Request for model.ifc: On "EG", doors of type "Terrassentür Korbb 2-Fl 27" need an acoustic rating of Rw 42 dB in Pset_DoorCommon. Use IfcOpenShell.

First a look at what the model holds.

```python
import ifcopenshell
import ifcopenshell.util.element

model = ifcopenshell.open("model.ifc")
print(model.schema)
storey = next(s for s in model.by_type("IfcBuildingStorey") if s.Name == "EG")
doors = [e for e in ifcopenshell.util.element.get_decomposition(storey) if e.is_a("IfcDoor")]
seen = {}
for e in doors:
    element_type = ifcopenshell.util.element.get_type(e)
    key = (element_type.Name if element_type != e and element_type else None, ifcopenshell.util.element.get_pset(e, "Pset_DoorCommon", "AcousticRating"))
    seen[key] = seen.get(key, 0) + 1
for (name, value), count in sorted(seen.items(), key=str):
    print(count, "x", name, "|", value)
```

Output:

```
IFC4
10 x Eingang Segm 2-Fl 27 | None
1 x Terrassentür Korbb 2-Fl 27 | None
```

```python
import ifcopenshell
import ifcopenshell.api.pset
import ifcopenshell.util.element

model = ifcopenshell.open("model.ifc")

storey = next(s for s in model.by_type("IfcBuildingStorey") if s.Name == "EG")
doors = [e for e in ifcopenshell.util.element.get_decomposition(storey) if e.is_a("IfcDoor")]

count = 0
for e in doors:
    element_type = ifcopenshell.util.element.get_type(e)
    if element_type in (None, e) or element_type.Name != "Terrassentür Korbb 2-Fl 27":
        continue
    # add_pset returns the element's existing set when there is one.
    pset = ifcopenshell.api.pset.add_pset(model, product=e, name="Pset_DoorCommon")
    ifcopenshell.api.pset.edit_pset(model, pset=pset, properties={"AcousticRating": "Rw 42 dB"})
    count += 1

print(count, "doors updated")

model.write("model_updated.ifc")
```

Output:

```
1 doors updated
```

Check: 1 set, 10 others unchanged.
